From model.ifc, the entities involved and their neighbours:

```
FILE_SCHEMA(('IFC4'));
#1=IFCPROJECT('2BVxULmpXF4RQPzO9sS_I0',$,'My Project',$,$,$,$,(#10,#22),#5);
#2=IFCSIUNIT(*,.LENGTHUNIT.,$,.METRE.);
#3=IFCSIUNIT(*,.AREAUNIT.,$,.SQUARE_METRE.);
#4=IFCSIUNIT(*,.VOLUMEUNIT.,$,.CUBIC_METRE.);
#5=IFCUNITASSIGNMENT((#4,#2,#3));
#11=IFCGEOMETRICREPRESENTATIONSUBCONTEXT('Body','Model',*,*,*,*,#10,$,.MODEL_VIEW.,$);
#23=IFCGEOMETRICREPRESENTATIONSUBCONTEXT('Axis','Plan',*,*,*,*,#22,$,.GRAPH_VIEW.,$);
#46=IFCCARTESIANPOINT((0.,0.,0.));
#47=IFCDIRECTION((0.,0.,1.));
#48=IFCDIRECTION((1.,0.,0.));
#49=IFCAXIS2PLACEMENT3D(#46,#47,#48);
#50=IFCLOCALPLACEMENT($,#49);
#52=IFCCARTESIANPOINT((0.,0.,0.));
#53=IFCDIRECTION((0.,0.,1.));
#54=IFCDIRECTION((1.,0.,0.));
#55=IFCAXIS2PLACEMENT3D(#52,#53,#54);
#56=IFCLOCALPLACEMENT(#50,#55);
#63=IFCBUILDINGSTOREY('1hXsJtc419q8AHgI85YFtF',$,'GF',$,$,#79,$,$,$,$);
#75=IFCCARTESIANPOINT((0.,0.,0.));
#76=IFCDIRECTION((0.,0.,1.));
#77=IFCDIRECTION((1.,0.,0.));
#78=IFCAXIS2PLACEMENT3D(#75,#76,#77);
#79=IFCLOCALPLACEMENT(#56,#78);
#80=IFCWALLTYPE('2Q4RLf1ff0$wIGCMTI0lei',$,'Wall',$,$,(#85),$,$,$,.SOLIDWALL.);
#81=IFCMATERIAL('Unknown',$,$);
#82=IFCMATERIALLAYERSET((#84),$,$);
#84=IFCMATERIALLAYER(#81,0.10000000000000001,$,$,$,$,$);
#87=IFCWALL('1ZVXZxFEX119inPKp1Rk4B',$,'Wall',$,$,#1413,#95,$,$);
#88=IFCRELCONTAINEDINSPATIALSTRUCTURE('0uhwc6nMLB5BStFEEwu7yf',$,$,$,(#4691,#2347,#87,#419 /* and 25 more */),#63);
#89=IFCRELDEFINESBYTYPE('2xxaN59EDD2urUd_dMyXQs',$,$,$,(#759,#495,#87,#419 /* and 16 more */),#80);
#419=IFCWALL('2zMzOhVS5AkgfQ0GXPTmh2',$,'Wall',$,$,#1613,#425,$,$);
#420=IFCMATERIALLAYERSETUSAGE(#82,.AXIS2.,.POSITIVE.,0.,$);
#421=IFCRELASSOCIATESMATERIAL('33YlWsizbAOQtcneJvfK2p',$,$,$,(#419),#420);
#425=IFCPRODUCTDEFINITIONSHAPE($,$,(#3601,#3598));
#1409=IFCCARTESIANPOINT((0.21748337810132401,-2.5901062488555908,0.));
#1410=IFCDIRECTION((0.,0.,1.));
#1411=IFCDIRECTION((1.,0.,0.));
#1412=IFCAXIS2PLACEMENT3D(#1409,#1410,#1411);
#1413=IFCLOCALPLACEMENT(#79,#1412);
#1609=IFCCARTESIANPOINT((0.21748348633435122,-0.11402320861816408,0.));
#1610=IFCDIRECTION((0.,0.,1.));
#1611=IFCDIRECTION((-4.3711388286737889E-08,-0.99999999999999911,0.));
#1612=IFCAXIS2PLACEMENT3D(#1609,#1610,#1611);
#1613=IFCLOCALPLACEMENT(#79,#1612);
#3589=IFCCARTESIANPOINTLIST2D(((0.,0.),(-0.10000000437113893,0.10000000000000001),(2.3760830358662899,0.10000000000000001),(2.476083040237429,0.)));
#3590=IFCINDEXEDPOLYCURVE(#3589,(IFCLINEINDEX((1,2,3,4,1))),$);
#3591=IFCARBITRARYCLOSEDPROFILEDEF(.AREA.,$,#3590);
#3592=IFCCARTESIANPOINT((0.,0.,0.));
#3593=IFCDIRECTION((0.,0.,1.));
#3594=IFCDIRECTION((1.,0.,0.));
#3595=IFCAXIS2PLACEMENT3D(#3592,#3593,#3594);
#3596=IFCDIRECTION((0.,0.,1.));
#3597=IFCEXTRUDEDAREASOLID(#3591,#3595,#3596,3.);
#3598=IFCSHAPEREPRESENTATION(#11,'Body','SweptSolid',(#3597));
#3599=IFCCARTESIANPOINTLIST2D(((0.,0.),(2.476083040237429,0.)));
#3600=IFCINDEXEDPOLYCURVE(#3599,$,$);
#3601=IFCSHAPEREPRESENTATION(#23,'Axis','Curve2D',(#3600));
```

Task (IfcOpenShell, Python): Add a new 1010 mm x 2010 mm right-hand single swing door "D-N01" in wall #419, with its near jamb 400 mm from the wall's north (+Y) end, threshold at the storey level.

```python
import numpy as np
import ifcopenshell
import ifcopenshell.api.feature
import ifcopenshell.api.geometry
import ifcopenshell.api.root
import ifcopenshell.api.spatial
import ifcopenshell.geom
import ifcopenshell.util.element
import ifcopenshell.util.placement
import ifcopenshell.util.representation
import ifcopenshell.util.shape
import ifcopenshell.util.unit

model = ifcopenshell.open("model.ifc")
unit_scale = ifcopenshell.util.unit.calculate_unit_scale(model)
settings = ifcopenshell.geom.settings()


def volume(element):
    """Net volume in cubic metres, openings subtracted."""
    shape = ifcopenshell.geom.create_shape(settings, element)
    return ifcopenshell.util.shape.get_volume(shape.geometry)


wall = model.by_guid("2zMzOhVS5AkgfQ0GXPTmh2")
storey = ifcopenshell.util.element.get_container(wall, ifc_class="IfcBuildingStorey")
context = ifcopenshell.util.representation.get_context(model, "Model", "Body", "MODEL_VIEW")
before = volume(wall)

width, height, from_end, sill = 1.01, 2.01, 0.4, 0.0  # metres

# The wall runs along its own X axis, and the end named is its -X end.
wall_shape = ifcopenshell.geom.create_shape(settings, wall)
x, y, z = ifcopenshell.util.shape.get_vertices(wall_shape.geometry).T
start = x.min() + from_end
face, thickness = float(y.min()), float(y.max() - y.min())
wall_matrix = ifcopenshell.util.placement.get_local_placement(wall.ObjectPlacement)
level = ifcopenshell.util.placement.get_local_placement(storey.ObjectPlacement)[2, 3]


def in_wall(x, y):
    """Placement at x, y metres in the wall's axes, at sill height."""
    matrix = wall_matrix.copy()
    matrix[:, 3] = wall_matrix @ np.array([x / unit_scale, y / unit_scale, 0.0, 1.0])
    matrix[2, 3] = level + sill / unit_scale
    return matrix


# Opening: a box that overshoots both wall faces by 50 mm.
opening = ifcopenshell.api.root.create_entity(model, ifc_class="IfcOpeningElement", predefined_type="OPENING")
box = ifcopenshell.api.geometry.add_wall_representation(
    model, context=context, length=width, height=height, thickness=thickness + 0.1
)
ifcopenshell.api.geometry.assign_representation(model, product=opening, representation=box)
ifcopenshell.api.geometry.edit_object_placement(model, product=opening, matrix=in_wall(start, face - 0.05), is_si=False)
ifcopenshell.api.feature.add_feature(model, feature=opening, element=wall)

door = ifcopenshell.api.root.create_entity(model, ifc_class="IfcDoor", name="D-N01", predefined_type="DOOR")
door.OverallWidth, door.OverallHeight = width / unit_scale, height / unit_scale
door.OperationType = "SINGLE_SWING_RIGHT"
body = ifcopenshell.api.geometry.add_door_representation(
    model,
    context=context,
    overall_width=door.OverallWidth,
    overall_height=door.OverallHeight,
    operation_type="SINGLE_SWING_RIGHT",
    lining_properties={"LiningDepth": thickness / unit_scale, "ThresholdDepth": thickness / unit_scale},
)
ifcopenshell.api.geometry.assign_representation(model, product=door, representation=body)
ifcopenshell.api.spatial.assign_container(model, products=[door], relating_structure=storey)
ifcopenshell.api.feature.add_filling(model, opening=opening, element=door)

# The lining spans the wall, so the door starts at the wall face.
ifcopenshell.api.geometry.edit_object_placement(model, product=door, matrix=in_wall(start, face), is_si=False)

after = volume(wall)

print(f"wall volume {before:.3f} -> {after:.3f} m3")

model.write("model_updated.ifc")
```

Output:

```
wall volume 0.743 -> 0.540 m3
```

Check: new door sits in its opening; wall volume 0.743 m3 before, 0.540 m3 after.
